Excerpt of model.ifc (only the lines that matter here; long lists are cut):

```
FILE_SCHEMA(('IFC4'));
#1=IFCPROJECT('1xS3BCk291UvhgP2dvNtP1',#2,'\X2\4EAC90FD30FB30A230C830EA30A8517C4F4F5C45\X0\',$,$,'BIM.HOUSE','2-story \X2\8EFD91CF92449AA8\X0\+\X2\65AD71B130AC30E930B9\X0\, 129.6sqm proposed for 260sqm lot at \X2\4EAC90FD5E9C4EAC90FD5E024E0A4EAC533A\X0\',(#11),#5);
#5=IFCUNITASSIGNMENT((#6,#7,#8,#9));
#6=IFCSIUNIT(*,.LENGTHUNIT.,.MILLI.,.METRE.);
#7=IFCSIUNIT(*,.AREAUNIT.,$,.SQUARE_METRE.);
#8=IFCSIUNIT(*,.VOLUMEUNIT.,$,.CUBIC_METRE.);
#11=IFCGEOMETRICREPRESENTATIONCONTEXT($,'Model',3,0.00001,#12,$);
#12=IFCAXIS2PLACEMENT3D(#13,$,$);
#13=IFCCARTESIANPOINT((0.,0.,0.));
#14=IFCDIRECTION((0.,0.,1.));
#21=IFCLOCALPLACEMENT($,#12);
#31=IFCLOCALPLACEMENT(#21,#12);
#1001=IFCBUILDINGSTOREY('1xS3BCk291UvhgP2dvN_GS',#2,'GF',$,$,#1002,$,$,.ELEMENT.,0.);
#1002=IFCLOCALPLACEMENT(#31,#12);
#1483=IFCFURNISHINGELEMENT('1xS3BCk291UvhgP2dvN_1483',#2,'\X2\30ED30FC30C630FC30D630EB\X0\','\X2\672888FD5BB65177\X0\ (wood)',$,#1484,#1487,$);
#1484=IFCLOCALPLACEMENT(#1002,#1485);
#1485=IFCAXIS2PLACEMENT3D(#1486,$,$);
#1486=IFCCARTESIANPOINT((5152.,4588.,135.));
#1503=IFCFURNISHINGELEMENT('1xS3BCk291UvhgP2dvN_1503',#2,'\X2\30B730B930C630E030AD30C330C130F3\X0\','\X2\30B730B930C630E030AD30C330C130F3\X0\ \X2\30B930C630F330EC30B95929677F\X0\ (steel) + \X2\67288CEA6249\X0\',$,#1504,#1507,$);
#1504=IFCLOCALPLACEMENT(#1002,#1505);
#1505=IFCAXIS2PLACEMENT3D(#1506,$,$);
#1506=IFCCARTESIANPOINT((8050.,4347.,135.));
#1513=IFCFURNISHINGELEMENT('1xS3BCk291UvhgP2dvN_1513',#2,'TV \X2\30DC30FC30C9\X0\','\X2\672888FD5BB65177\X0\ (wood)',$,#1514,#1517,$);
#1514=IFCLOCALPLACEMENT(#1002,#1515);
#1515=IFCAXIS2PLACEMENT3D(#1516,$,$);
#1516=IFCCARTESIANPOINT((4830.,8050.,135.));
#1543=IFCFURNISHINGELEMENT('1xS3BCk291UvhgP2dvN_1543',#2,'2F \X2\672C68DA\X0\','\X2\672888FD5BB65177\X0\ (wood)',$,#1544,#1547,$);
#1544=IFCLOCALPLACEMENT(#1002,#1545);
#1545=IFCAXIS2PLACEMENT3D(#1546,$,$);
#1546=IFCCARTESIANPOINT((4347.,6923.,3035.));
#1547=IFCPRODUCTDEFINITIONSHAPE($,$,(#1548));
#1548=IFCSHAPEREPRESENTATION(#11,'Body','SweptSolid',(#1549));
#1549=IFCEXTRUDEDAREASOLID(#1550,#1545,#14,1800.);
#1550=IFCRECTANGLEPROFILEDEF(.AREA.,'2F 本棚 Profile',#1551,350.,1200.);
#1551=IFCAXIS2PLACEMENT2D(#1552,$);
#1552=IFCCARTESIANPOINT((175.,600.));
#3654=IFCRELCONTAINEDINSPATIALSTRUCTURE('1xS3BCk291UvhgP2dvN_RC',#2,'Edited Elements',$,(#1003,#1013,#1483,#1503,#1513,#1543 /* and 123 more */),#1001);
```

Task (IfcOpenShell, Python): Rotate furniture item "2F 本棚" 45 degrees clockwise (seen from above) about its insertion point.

```python
import ifcopenshell
import ifcopenshell.api.geometry
import ifcopenshell.util.placement

model = ifcopenshell.open("model.ifc")

item = model.by_id(1543)
matrix = ifcopenshell.util.placement.get_local_placement(item.ObjectPlacement)
matrix = matrix @ ifcopenshell.util.placement.rotation(-45, "Z")
ifcopenshell.api.geometry.edit_object_placement(model, product=item, matrix=matrix, is_si=False)

print(ifcopenshell.util.placement.get_local_placement(item.ObjectPlacement).round(3) + 0.0)

model.write("model_v2.ifc")
```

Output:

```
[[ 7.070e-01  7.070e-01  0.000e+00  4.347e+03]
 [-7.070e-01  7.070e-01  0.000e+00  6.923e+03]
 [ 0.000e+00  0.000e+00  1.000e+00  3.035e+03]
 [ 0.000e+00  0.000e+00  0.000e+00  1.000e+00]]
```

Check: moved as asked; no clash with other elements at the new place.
